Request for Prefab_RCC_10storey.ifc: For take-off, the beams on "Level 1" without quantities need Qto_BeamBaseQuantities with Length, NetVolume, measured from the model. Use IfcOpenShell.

First a look at what the model holds.

```python
import ifcopenshell
import ifcopenshell.util.element
import ifcopenshell.util.unit

model = ifcopenshell.open("Prefab_RCC_10storey.ifc")
print(model.schema)
for unit_type in ("LENGTHUNIT", "AREAUNIT", "VOLUMEUNIT"):
    print(unit_type, ifcopenshell.util.unit.calculate_unit_scale(model, unit_type))
storey = next(s for s in model.by_type("IfcBuildingStorey") if s.Name == "Level 1")
beams = [e for e in ifcopenshell.util.element.get_decomposition(storey) if e.is_a("IfcBeam")]
for e in sorted(beams, key=lambda e: e.id()):
    print(e.id(), e.is_a(), e.Name, list(ifcopenshell.util.element.get_psets(e, qtos_only=True)), sep=" | ")
```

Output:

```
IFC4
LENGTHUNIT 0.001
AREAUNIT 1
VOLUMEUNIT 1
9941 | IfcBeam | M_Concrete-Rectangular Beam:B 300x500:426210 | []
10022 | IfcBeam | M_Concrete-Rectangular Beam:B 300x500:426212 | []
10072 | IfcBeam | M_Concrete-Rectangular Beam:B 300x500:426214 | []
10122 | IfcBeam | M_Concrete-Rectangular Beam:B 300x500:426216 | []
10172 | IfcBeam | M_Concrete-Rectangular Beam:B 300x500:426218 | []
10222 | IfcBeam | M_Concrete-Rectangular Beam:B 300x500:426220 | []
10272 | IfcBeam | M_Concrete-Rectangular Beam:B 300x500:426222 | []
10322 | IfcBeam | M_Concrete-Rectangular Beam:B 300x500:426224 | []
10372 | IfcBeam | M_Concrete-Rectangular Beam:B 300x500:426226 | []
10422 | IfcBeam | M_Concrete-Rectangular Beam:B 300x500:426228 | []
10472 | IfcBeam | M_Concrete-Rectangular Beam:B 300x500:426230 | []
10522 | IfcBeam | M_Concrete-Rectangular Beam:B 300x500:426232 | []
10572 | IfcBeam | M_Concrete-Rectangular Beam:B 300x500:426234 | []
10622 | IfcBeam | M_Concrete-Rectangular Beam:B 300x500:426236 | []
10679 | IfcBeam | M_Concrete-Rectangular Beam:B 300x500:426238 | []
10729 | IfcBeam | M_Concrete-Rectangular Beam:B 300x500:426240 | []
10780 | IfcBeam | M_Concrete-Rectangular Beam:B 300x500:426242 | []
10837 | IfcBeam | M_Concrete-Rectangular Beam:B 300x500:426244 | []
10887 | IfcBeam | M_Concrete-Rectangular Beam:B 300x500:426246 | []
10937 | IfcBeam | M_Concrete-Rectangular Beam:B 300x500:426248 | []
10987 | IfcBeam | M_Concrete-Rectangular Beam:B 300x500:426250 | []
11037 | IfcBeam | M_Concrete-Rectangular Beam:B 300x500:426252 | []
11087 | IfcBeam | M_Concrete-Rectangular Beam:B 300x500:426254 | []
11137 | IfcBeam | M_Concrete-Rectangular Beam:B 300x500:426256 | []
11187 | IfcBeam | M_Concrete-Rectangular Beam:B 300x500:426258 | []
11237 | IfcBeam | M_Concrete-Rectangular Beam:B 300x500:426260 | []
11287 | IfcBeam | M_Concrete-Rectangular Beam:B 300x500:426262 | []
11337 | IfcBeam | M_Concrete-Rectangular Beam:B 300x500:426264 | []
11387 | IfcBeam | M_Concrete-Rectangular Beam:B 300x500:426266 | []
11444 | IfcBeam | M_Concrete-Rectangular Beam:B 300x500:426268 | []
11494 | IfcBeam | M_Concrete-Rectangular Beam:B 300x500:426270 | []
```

```python
import ifcopenshell
import ifcopenshell.api.pset
import ifcopenshell.geom
import ifcopenshell.util.element
import ifcopenshell.util.shape
import ifcopenshell.util.unit

model = ifcopenshell.open("Prefab_RCC_10storey.ifc")
unit_scale = ifcopenshell.util.unit.calculate_unit_scale(model)
volume_scale = ifcopenshell.util.unit.calculate_unit_scale(model, "VOLUMEUNIT")
settings = ifcopenshell.geom.settings()

storey = next(s for s in model.by_type("IfcBuildingStorey") if s.Name == "Level 1")
beams = [e for e in ifcopenshell.util.element.get_decomposition(storey) if e.is_a("IfcBeam")]

for e in sorted(beams, key=lambda e: e.id()):
    if ifcopenshell.util.element.get_psets(e, qtos_only=True, should_inherit=False):
        continue
    # Geometry comes back in metres, in the element's own axes.
    shape = ifcopenshell.geom.create_shape(settings, e)
    values = {
        "Length": ifcopenshell.util.shape.get_max_xyz(shape.geometry) / unit_scale,
        "NetVolume": ifcopenshell.util.shape.get_volume(shape.geometry) / volume_scale,
    }
    qto = ifcopenshell.api.pset.add_qto(model, product=e, name="Qto_BeamBaseQuantities")
    ifcopenshell.api.pset.edit_qto(model, qto=qto, properties=values)
    print(e.id(), {k: round(v, 3) for k, v in values.items()})

model.write("Prefab_RCC_10storey_v2.ifc")
```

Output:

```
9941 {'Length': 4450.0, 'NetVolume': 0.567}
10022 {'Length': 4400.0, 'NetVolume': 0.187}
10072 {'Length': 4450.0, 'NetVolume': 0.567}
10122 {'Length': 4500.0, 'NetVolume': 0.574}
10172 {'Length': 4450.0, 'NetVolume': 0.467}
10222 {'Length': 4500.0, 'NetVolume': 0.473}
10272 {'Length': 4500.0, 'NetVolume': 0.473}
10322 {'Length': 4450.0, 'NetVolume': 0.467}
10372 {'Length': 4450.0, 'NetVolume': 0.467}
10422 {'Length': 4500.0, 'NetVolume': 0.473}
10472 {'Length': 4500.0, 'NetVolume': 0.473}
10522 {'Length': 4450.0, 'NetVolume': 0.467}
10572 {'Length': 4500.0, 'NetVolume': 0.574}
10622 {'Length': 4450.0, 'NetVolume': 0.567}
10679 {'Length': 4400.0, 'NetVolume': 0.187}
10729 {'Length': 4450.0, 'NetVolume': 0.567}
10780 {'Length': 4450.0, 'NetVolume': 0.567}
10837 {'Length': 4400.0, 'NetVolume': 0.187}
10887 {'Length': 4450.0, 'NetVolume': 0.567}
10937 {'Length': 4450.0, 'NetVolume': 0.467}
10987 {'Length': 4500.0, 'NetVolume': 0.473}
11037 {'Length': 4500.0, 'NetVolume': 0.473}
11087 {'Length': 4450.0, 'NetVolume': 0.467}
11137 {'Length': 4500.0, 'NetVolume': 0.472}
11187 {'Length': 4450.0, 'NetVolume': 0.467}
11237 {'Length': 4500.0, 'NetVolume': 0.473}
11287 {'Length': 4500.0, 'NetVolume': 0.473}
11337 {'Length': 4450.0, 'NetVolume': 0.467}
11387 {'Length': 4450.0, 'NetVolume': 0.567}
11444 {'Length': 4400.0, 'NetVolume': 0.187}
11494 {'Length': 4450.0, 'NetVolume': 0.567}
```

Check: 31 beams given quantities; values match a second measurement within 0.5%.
